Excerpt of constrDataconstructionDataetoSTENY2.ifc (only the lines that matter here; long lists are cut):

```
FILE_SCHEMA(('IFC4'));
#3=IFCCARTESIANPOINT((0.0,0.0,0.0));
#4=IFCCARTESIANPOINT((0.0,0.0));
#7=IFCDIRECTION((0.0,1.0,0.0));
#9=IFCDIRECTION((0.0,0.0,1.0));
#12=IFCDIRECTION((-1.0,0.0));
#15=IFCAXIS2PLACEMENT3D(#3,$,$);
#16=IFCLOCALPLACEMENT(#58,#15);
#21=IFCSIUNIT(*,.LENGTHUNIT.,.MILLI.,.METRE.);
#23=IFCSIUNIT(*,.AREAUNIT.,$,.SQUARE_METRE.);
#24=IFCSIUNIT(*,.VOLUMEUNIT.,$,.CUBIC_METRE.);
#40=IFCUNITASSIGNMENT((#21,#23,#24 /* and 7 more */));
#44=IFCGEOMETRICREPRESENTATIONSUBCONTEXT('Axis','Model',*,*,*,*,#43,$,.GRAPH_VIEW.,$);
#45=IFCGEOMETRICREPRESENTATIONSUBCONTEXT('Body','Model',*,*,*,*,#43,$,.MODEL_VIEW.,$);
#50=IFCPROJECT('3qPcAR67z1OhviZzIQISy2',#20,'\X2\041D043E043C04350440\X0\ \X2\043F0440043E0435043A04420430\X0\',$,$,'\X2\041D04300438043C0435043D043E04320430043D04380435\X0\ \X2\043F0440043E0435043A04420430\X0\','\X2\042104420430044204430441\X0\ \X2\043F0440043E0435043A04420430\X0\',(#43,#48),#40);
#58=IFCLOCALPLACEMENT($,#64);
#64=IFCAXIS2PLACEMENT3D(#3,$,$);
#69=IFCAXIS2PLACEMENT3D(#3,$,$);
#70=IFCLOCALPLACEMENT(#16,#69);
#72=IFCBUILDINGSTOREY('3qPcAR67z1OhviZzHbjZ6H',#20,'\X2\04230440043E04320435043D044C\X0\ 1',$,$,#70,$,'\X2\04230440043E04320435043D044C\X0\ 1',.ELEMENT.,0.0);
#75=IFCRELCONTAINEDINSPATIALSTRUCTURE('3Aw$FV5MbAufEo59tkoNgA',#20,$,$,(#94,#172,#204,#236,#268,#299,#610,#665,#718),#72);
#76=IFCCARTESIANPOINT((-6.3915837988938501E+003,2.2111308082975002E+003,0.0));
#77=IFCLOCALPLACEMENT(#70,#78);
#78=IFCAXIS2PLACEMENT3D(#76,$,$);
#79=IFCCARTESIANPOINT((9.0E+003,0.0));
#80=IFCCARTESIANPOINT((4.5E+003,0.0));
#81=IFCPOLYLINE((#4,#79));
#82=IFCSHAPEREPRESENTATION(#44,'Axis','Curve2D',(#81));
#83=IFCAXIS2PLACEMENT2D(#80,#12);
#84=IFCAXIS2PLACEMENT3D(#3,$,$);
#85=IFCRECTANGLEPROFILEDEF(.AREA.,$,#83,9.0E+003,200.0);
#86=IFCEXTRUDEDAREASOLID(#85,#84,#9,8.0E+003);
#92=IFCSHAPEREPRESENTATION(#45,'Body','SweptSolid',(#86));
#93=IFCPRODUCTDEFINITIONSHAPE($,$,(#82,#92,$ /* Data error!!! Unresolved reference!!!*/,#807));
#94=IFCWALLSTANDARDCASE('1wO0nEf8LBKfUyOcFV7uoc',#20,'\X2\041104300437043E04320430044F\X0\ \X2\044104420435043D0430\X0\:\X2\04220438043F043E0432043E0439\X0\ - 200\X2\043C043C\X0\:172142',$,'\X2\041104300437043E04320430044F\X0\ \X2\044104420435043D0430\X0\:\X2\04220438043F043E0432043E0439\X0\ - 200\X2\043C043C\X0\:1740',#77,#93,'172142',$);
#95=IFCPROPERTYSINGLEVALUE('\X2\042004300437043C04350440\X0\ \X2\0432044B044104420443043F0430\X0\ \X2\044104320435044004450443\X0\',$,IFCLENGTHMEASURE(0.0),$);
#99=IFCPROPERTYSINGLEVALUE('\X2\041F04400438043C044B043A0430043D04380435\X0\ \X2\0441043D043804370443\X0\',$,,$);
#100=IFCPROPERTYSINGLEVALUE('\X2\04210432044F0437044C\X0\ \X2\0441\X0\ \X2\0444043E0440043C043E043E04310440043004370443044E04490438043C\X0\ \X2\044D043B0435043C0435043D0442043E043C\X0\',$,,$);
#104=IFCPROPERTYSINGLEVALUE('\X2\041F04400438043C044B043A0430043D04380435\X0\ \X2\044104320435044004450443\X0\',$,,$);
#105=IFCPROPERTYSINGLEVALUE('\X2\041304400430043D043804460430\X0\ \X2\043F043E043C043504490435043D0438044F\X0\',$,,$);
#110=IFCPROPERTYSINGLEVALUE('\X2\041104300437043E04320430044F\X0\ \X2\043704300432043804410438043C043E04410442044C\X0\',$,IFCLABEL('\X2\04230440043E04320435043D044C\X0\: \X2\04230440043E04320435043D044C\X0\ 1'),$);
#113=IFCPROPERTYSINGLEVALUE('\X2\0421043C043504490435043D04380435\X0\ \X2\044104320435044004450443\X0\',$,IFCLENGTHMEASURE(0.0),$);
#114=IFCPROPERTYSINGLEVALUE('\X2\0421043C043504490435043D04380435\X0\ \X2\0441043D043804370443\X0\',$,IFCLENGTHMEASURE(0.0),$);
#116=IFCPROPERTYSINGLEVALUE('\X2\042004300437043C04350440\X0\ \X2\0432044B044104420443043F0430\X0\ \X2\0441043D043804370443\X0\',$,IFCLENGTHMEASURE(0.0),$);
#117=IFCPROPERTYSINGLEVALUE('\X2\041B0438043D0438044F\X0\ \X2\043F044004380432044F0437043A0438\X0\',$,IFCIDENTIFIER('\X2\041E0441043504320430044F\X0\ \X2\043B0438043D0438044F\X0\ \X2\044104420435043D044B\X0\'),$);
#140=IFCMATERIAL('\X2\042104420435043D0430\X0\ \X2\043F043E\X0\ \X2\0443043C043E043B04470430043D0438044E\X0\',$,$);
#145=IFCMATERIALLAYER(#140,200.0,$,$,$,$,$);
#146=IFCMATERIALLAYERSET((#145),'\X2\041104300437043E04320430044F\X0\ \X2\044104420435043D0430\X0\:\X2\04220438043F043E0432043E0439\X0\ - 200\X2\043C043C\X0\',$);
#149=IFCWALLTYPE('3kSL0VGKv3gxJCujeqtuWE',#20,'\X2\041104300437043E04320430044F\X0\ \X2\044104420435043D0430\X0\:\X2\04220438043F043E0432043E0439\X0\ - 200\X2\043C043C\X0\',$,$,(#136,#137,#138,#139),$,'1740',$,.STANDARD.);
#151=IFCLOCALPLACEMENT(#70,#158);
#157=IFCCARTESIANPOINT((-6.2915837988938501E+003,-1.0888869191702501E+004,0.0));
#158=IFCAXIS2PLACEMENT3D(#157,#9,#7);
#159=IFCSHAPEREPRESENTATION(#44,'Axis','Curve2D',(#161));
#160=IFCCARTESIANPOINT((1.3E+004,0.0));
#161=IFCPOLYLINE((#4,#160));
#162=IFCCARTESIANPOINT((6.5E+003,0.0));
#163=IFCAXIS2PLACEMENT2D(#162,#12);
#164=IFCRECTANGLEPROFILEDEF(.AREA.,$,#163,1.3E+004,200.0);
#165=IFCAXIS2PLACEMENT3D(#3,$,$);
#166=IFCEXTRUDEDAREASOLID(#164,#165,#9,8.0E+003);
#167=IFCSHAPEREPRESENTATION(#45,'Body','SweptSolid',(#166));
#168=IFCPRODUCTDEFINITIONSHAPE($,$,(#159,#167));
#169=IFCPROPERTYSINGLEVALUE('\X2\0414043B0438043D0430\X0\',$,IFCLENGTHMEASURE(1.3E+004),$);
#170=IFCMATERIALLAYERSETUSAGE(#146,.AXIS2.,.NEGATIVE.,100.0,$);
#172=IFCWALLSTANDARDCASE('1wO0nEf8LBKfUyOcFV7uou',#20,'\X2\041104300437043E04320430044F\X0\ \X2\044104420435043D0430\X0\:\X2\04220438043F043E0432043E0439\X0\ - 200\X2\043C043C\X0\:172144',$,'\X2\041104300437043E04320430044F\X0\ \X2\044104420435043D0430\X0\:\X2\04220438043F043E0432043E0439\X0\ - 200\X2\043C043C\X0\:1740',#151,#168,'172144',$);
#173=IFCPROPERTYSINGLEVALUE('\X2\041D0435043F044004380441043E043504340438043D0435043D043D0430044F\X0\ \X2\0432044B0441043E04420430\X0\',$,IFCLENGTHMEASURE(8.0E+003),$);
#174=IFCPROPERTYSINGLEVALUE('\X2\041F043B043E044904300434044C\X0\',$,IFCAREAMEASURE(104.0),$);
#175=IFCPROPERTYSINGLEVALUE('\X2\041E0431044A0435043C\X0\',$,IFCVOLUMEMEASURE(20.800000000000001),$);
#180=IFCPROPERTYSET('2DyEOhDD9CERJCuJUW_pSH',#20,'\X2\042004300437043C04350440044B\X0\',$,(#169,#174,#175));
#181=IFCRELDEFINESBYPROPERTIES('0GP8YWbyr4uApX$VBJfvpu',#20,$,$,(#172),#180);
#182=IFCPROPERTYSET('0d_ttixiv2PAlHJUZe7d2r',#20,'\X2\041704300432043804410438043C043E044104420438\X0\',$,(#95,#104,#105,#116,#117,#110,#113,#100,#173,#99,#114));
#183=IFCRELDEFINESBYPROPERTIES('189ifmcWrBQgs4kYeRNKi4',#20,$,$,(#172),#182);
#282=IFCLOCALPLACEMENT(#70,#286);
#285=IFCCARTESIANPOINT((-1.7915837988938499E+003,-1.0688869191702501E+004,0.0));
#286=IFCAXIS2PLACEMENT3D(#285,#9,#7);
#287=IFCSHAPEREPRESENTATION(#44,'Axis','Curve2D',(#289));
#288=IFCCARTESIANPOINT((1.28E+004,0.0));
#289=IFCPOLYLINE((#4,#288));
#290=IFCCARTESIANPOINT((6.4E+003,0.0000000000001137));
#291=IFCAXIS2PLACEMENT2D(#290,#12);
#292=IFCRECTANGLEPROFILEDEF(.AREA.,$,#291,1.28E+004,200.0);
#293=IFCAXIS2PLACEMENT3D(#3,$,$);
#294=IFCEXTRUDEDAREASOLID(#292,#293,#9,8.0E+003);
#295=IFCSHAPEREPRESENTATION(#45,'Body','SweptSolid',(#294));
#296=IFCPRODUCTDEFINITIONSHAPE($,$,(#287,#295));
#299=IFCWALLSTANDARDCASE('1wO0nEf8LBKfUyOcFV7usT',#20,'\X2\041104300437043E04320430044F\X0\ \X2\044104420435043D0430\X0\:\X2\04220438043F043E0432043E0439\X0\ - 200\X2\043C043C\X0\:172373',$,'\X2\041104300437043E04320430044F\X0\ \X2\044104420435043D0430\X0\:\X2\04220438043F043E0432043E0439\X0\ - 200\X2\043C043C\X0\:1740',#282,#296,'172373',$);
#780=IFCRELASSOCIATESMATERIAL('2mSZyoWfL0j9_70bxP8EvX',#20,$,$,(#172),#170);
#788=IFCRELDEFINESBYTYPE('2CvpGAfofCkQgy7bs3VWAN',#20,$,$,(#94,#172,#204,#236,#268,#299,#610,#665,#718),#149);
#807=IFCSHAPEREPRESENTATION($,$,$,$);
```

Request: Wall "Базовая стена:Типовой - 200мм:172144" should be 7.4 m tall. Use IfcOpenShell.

```python
import ifcopenshell
import ifcopenshell.api.pset
import ifcopenshell.geom
import ifcopenshell.util.element
import ifcopenshell.util.representation
import ifcopenshell.util.shape
import ifcopenshell.util.unit

model = ifcopenshell.open("constrDataconstructionDataetoSTENY2.ifc")
area_scale = ifcopenshell.util.unit.calculate_unit_scale(model, "AREAUNIT")
volume_scale = ifcopenshell.util.unit.calculate_unit_scale(model, "VOLUMEUNIT")
settings = ifcopenshell.geom.settings()


def volume(element):
    """Net volume in cubic metres, openings subtracted."""
    shape = ifcopenshell.geom.create_shape(settings, element)
    return ifcopenshell.util.shape.get_volume(shape.geometry)


wall = model.by_guid("1wO0nEf8LBKfUyOcFV7uou")
before = volume(wall)

body = ifcopenshell.util.representation.get_representation(wall, "Model", "Body")
solid = body.Items[0]
old_height = solid.Depth
solid.Depth = 7400.0
after = volume(wall)
thickness = 0.2  # wall thickness in metres

# Update the stored height, areas and volumes.
pset = model.by_id(ifcopenshell.util.element.get_pset(wall, "Размеры", should_inherit=False)["id"])
ifcopenshell.api.pset.edit_pset(model, pset=pset, properties={
    "Площадь": model.create_entity("IfcAreaMeasure", after / thickness / area_scale),
    "Объем": model.create_entity("IfcVolumeMeasure", after / volume_scale),
})
pset = model.by_id(ifcopenshell.util.element.get_pset(wall, "Зависимости", should_inherit=False)["id"])
ifcopenshell.api.pset.edit_pset(model, pset=pset, properties={
    "Неприсоединенная высота": model.create_entity("IfcLengthMeasure", solid.Depth),
})

print(f"height {old_height:g} -> {solid.Depth:g}, volume {before:.3f} -> {after:.3f} m3")

model.write("constrDataconstructionDataetoSTENY2_v2.ifc")
```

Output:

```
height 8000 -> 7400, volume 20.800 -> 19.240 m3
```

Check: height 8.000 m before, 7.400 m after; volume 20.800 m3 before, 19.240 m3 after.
